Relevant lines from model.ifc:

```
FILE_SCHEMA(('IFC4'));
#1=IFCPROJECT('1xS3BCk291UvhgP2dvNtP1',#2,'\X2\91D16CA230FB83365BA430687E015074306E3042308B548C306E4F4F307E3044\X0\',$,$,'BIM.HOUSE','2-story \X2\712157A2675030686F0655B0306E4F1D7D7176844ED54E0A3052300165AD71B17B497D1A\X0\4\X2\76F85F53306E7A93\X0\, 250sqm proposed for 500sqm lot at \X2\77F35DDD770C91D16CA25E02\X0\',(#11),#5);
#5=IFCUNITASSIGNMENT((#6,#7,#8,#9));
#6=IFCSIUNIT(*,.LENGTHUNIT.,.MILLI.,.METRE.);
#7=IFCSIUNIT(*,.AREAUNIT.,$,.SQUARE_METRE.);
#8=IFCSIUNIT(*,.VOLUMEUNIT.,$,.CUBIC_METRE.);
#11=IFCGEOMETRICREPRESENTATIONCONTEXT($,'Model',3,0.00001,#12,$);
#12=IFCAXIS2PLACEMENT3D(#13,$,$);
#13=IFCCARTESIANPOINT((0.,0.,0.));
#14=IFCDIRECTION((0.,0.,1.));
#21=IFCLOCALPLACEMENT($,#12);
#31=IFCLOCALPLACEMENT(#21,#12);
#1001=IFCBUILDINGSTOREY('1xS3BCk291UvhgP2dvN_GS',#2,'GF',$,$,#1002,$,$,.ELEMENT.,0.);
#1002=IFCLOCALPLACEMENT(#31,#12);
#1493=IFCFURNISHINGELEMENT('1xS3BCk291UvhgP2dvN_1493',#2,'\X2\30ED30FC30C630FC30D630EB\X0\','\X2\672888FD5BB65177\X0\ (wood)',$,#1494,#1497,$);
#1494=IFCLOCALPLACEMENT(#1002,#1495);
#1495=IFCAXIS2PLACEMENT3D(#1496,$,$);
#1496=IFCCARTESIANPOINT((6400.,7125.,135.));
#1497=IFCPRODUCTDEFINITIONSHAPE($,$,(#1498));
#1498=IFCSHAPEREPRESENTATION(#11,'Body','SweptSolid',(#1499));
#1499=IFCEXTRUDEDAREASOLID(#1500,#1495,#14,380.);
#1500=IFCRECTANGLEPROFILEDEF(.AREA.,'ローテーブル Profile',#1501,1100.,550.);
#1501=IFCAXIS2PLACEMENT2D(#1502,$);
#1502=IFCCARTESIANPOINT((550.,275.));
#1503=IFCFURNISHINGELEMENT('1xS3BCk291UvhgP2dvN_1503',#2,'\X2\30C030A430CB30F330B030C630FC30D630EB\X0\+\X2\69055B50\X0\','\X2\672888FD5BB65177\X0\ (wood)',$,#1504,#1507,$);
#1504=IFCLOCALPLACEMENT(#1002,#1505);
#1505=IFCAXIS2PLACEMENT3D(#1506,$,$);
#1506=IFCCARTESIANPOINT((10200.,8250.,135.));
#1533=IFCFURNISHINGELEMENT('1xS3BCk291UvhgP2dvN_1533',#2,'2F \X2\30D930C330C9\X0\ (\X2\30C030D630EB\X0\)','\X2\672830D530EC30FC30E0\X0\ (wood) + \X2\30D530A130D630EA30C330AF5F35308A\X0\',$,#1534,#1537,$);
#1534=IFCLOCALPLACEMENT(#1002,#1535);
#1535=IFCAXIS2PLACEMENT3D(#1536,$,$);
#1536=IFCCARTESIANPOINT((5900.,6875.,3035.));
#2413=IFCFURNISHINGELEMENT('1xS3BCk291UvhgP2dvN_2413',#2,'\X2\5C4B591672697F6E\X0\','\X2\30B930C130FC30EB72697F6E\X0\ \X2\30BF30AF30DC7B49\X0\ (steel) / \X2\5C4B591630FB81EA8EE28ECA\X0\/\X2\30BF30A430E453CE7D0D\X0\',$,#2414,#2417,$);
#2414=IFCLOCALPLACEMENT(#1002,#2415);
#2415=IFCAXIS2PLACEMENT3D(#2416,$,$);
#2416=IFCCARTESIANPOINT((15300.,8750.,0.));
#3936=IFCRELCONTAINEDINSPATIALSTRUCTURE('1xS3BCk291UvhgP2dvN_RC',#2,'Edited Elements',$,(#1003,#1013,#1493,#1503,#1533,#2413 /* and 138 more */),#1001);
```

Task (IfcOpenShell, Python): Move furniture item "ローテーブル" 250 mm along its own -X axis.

```python
import ifcopenshell
import ifcopenshell.api.geometry
import ifcopenshell.util.placement

model = ifcopenshell.open("model.ifc")

item = model.by_id(1493)
matrix = ifcopenshell.util.placement.get_local_placement(item.ObjectPlacement)
matrix[:3, 3] -= matrix[:3, 0] * 250.0
ifcopenshell.api.geometry.edit_object_placement(model, product=item, matrix=matrix, is_si=False)

print(ifcopenshell.util.placement.get_local_placement(item.ObjectPlacement).round(3) + 0.0)

model.write("model_v2.ifc")
```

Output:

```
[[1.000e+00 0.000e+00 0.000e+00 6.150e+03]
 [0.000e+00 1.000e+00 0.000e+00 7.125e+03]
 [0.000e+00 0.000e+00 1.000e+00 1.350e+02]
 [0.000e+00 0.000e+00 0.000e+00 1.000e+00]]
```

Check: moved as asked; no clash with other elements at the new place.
